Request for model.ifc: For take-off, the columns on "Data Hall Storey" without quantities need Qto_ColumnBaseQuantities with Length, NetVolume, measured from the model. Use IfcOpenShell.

First a look at what the model holds.

```python
import ifcopenshell
import ifcopenshell.util.element
import ifcopenshell.util.unit

model = ifcopenshell.open("model.ifc")
print(model.schema)
for unit_type in ("LENGTHUNIT", "AREAUNIT", "VOLUMEUNIT"):
    print(unit_type, ifcopenshell.util.unit.calculate_unit_scale(model, unit_type))
storey = next(s for s in model.by_type("IfcBuildingStorey") if s.Name == "Data Hall Storey")
columns = [e for e in ifcopenshell.util.element.get_decomposition(storey) if e.is_a("IfcColumn")]
for e in sorted(columns, key=lambda e: e.id()):
    print(e.id(), e.is_a(), e.Name, list(ifcopenshell.util.element.get_psets(e, qtos_only=True)), sep=" | ")
```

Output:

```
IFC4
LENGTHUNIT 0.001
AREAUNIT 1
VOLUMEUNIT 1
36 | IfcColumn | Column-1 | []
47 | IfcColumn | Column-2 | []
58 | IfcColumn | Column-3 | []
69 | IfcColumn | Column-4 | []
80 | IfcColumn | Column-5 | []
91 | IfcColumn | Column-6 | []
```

```python
import ifcopenshell
import ifcopenshell.api.pset
import ifcopenshell.geom
import ifcopenshell.util.element
import ifcopenshell.util.shape
import ifcopenshell.util.unit

model = ifcopenshell.open("model.ifc")
unit_scale = ifcopenshell.util.unit.calculate_unit_scale(model)
volume_scale = ifcopenshell.util.unit.calculate_unit_scale(model, "VOLUMEUNIT")
settings = ifcopenshell.geom.settings()

storey = next(s for s in model.by_type("IfcBuildingStorey") if s.Name == "Data Hall Storey")
columns = [e for e in ifcopenshell.util.element.get_decomposition(storey) if e.is_a("IfcColumn")]

for e in sorted(columns, key=lambda e: e.id()):
    if ifcopenshell.util.element.get_psets(e, qtos_only=True, should_inherit=False):
        continue
    # Geometry comes back in metres, in the element's own axes.
    shape = ifcopenshell.geom.create_shape(settings, e)
    values = {
        "Length": ifcopenshell.util.shape.get_z(shape.geometry) / unit_scale,
        "NetVolume": ifcopenshell.util.shape.get_volume(shape.geometry) / volume_scale,
    }
    qto = ifcopenshell.api.pset.add_qto(model, product=e, name="Qto_ColumnBaseQuantities")
    ifcopenshell.api.pset.edit_qto(model, qto=qto, properties=values)
    print(e.id(), {k: round(v, 3) for k, v in values.items()})

model.write("model_edited.ifc")
```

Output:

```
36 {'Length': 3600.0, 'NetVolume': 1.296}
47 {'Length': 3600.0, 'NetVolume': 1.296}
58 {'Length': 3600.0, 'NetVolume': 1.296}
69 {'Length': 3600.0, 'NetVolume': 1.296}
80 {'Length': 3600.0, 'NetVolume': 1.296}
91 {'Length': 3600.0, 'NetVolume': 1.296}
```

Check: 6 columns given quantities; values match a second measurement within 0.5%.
